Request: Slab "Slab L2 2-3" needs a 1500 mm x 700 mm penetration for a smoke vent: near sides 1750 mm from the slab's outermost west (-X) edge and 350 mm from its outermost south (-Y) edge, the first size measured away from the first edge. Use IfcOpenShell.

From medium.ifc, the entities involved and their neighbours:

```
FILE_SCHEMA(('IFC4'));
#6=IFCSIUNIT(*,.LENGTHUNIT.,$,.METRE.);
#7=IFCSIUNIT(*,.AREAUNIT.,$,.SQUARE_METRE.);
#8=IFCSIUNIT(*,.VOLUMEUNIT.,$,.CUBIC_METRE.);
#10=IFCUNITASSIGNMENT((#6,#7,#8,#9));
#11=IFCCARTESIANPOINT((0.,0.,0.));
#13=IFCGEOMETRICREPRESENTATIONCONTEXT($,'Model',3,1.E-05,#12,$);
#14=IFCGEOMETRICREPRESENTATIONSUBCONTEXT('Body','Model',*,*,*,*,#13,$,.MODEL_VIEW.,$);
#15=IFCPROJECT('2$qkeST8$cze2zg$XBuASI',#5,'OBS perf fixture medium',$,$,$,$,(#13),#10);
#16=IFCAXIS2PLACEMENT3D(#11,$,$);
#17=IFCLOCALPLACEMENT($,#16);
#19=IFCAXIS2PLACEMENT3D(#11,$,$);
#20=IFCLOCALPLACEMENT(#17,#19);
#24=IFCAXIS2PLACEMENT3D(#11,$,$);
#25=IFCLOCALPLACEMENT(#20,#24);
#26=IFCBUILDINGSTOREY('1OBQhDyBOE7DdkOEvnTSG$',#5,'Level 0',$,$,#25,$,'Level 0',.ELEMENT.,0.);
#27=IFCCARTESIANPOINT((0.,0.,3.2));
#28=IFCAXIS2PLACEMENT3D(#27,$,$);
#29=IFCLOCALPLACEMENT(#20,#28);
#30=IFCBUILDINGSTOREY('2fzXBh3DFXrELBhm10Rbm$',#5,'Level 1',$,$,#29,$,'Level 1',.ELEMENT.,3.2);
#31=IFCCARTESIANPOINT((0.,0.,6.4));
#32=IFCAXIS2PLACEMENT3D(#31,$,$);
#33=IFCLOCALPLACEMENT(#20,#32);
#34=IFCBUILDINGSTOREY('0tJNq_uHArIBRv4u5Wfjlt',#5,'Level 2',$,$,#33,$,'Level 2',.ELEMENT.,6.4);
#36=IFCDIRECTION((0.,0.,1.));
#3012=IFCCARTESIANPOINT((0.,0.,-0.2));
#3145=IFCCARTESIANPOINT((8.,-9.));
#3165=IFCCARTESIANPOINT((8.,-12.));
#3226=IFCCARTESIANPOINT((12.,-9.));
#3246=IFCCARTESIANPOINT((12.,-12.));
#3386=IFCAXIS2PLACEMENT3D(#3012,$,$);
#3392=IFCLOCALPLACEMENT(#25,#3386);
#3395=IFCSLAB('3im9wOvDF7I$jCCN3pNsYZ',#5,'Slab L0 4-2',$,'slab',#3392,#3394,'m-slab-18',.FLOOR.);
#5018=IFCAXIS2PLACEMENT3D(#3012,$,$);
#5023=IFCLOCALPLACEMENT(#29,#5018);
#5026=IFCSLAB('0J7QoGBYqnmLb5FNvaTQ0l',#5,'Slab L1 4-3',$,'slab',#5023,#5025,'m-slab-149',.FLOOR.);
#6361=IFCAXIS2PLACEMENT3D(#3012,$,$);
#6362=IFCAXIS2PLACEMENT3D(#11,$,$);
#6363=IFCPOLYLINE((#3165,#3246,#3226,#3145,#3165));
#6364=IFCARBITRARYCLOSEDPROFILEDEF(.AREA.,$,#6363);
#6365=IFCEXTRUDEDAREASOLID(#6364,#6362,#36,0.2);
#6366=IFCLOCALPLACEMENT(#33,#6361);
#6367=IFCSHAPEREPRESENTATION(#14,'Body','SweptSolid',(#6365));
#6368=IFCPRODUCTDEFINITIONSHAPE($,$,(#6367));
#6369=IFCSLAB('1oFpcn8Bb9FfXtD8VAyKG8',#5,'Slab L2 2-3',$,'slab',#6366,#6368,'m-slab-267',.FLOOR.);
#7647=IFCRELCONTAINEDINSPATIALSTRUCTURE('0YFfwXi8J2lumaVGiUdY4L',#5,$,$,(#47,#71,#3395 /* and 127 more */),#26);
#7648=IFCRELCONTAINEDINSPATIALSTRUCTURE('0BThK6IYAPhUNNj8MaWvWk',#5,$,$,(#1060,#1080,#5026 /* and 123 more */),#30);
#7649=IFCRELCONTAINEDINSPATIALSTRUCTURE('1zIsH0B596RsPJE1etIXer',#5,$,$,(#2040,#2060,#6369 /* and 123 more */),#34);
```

```python
import numpy as np
import ifcopenshell
import ifcopenshell.api.feature
import ifcopenshell.api.geometry
import ifcopenshell.api.root
import ifcopenshell.geom
import ifcopenshell.util.placement
import ifcopenshell.util.representation
import ifcopenshell.util.shape
import ifcopenshell.util.unit

model = ifcopenshell.open("medium.ifc")
unit_scale = ifcopenshell.util.unit.calculate_unit_scale(model)
settings = ifcopenshell.geom.settings()


def volume(element):
    """Net volume in cubic metres, openings subtracted."""
    shape = ifcopenshell.geom.create_shape(settings, element)
    return ifcopenshell.util.shape.get_volume(shape.geometry)


slab = model.by_id(6369)
before = volume(slab)

# Extent in the slab's own axes, in metres. The edges named are its -X and -Y sides.
slab_shape = ifcopenshell.geom.create_shape(settings, slab)
vertices = ifcopenshell.util.shape.get_vertices(slab_shape.geometry)
x_min, y_min, bottom = vertices.min(axis=0)
top = vertices[:, 2].max()

opening = ifcopenshell.api.root.create_entity(model, ifc_class="IfcOpeningElement", name="Smoke vent opening", predefined_type="OPENING")
context = ifcopenshell.util.representation.get_context(model, "Model", "Body", "MODEL_VIEW")
width, depth = 1.5, 0.7
outline = [(0.0, 0.0), (width, 0.0), (width, depth), (0.0, depth), (0.0, 0.0)]
# Overshoot both faces by 50 mm so the cut is clean.
shape = ifcopenshell.api.geometry.add_slab_representation(
    model, context=context, depth=top - bottom + 0.1, polyline=outline
)
ifcopenshell.api.geometry.assign_representation(model, product=opening, representation=shape)

matrix = ifcopenshell.util.placement.get_local_placement(slab.ObjectPlacement)
matrix[:, 3] = matrix @ np.append(np.array([x_min + 1.75, y_min + 0.35, bottom - 0.05]) / unit_scale, 1.0)
ifcopenshell.api.geometry.edit_object_placement(model, product=opening, matrix=matrix, is_si=False)
ifcopenshell.api.feature.add_feature(model, feature=opening, element=slab)

after = volume(slab)

print(f"slab volume {before:.3f} -> {after:.3f} m3")

model.write("medium-out.ifc")
```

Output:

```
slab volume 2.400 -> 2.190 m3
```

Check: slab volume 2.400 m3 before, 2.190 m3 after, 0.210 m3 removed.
